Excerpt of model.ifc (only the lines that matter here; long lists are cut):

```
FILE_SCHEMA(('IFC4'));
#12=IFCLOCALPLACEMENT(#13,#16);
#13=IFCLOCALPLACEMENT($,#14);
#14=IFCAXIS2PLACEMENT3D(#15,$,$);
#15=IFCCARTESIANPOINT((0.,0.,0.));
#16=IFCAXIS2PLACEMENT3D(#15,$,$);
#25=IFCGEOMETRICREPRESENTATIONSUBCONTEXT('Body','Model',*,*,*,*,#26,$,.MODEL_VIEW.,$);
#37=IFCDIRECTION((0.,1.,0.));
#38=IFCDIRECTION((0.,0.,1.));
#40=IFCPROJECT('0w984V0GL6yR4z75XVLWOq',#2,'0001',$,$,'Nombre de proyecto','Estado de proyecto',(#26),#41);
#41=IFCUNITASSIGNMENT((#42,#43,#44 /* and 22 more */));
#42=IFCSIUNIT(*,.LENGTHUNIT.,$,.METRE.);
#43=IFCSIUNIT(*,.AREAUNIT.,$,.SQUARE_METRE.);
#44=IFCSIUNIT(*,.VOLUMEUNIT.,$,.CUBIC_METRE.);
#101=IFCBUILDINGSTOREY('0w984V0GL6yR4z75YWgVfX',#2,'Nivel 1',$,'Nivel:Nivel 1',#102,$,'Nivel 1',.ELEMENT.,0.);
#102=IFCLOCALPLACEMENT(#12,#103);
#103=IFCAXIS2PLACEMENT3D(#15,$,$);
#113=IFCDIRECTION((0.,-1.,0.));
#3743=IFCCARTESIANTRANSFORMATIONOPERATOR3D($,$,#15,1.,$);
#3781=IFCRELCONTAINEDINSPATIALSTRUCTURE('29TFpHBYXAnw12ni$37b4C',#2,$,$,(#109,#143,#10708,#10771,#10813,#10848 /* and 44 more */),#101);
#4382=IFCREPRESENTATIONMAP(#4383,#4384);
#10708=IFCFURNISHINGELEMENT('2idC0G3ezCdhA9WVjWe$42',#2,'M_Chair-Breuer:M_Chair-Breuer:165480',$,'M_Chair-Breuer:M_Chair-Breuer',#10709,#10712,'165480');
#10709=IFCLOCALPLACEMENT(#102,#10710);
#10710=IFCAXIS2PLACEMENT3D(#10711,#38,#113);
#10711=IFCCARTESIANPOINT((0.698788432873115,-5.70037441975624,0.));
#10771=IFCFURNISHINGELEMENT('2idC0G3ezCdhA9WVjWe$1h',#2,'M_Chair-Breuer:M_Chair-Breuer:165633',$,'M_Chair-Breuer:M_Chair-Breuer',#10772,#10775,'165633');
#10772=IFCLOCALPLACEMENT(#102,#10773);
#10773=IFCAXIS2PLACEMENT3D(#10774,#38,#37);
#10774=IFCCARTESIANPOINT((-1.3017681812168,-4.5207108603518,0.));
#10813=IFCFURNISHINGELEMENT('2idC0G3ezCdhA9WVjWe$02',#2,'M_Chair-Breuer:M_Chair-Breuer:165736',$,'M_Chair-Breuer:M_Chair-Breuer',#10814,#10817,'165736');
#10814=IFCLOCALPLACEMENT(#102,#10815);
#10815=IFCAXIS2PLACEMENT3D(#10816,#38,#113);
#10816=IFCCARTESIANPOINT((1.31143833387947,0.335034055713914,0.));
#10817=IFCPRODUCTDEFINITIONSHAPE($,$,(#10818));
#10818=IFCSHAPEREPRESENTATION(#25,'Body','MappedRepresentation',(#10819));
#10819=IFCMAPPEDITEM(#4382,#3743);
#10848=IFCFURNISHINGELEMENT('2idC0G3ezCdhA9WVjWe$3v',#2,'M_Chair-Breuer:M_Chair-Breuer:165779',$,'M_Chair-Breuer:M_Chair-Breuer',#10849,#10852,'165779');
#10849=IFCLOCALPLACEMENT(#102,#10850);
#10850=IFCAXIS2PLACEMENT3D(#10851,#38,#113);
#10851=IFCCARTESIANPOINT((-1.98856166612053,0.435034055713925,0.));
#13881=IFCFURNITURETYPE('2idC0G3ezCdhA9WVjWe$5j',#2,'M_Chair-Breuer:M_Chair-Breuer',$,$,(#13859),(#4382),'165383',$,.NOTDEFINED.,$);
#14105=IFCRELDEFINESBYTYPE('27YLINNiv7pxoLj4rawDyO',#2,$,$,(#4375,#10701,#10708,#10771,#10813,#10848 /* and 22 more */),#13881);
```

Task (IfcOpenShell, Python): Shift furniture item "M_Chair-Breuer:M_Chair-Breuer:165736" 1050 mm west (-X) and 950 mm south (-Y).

```python
import ifcopenshell
import ifcopenshell.api.geometry
import ifcopenshell.util.placement

model = ifcopenshell.open("model.ifc")

item = model.by_guid("2idC0G3ezCdhA9WVjWe$02")
matrix = ifcopenshell.util.placement.get_local_placement(item.ObjectPlacement)
matrix[0, 3] -= 1.05
matrix[1, 3] -= 0.95
ifcopenshell.api.geometry.edit_object_placement(model, product=item, matrix=matrix, is_si=False)

print(ifcopenshell.util.placement.get_local_placement(item.ObjectPlacement).round(3) + 0.0)

model.write("model_rev.ifc")
```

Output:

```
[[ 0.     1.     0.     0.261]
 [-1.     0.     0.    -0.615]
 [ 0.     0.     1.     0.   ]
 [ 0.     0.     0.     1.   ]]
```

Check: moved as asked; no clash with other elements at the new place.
